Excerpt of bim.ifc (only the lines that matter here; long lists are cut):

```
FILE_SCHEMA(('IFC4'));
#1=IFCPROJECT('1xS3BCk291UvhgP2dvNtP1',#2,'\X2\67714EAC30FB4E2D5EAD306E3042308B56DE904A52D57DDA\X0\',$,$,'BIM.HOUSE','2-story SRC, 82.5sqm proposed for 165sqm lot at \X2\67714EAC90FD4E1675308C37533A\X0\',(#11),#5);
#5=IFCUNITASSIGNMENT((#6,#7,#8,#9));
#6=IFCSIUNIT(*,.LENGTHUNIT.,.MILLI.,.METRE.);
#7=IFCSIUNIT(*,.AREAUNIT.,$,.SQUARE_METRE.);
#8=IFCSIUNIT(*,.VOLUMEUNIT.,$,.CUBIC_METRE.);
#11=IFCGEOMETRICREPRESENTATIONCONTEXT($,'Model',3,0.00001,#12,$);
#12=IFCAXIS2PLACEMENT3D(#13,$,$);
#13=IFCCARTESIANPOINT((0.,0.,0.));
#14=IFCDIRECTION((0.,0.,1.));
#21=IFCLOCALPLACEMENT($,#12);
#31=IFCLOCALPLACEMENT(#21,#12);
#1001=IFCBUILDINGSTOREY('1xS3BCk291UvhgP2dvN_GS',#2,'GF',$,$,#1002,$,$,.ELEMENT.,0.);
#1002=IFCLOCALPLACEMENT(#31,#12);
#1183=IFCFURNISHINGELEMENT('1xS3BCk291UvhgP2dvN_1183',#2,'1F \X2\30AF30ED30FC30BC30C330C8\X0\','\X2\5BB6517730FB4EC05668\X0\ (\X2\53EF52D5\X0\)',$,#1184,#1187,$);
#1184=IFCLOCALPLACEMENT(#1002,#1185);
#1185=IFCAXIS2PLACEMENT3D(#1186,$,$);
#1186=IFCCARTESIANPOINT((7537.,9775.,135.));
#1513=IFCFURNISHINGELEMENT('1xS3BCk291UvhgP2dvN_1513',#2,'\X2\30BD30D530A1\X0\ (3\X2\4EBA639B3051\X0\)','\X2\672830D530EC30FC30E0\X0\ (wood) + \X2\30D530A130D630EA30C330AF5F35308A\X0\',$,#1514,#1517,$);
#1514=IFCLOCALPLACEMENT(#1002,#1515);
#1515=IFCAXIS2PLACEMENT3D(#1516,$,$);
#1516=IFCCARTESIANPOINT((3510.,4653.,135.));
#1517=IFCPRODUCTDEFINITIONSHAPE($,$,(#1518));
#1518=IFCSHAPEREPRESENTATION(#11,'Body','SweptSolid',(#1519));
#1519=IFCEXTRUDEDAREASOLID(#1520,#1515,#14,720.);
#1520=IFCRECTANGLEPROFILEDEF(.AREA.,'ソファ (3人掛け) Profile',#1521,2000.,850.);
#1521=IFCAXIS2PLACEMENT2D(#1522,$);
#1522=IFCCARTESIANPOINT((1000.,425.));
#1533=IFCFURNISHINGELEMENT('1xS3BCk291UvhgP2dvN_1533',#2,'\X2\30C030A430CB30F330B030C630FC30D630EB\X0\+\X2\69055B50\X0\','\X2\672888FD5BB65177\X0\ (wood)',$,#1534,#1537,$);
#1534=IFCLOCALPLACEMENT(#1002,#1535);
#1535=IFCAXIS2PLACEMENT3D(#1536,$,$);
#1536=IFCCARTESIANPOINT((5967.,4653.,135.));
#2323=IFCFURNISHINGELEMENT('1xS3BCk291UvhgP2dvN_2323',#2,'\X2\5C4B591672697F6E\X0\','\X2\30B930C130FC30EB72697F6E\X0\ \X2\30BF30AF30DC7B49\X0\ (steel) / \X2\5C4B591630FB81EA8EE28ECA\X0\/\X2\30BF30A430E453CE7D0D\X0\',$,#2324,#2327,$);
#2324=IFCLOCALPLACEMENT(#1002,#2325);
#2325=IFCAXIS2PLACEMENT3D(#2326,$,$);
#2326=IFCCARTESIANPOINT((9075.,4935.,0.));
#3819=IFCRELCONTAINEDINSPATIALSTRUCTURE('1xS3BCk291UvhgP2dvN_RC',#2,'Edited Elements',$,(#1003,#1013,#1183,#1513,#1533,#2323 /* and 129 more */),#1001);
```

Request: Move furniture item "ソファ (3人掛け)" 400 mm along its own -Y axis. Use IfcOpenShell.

```python
import ifcopenshell
import ifcopenshell.api.geometry
import ifcopenshell.util.placement

model = ifcopenshell.open("bim.ifc")

item = model.by_guid("1xS3BCk291UvhgP2dvN_1513")
matrix = ifcopenshell.util.placement.get_local_placement(item.ObjectPlacement)
matrix[:3, 3] -= matrix[:3, 1] * 400.0
ifcopenshell.api.geometry.edit_object_placement(model, product=item, matrix=matrix, is_si=False)

print(ifcopenshell.util.placement.get_local_placement(item.ObjectPlacement).round(3) + 0.0)

model.write("bim-out.ifc")
```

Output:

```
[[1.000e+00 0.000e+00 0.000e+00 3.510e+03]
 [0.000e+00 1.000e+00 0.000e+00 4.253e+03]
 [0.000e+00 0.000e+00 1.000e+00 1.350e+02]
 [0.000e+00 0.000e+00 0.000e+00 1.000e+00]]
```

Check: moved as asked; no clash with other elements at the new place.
